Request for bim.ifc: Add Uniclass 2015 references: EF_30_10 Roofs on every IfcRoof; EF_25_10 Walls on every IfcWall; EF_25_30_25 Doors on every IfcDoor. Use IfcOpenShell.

First a look at what the model holds.

```python
import ifcopenshell

model = ifcopenshell.open("bim.ifc")
print(model.schema)
print("classifications:", [c.Name for c in model.by_type("IfcClassification")])
for ifc_class in ("IfcDoor", "IfcRoof", "IfcStair", "IfcWall", "IfcWindow"):
    print(ifc_class, len(model.by_type(ifc_class)))
```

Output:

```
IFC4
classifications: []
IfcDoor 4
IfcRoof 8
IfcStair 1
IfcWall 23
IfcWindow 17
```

```python
import ifcopenshell
import ifcopenshell.api.classification

model = ifcopenshell.open("bim.ifc")

system = ifcopenshell.api.classification.add_classification(model, classification="Uniclass 2015")

codes = {
    "IfcRoof": ("EF_30_10", "Roofs"),
    "IfcWall": ("EF_25_10", "Walls"),
    "IfcDoor": ("EF_25_30_25", "Doors"),
}
for ifc_class, (code, name) in codes.items():
    products = model.by_type(ifc_class)
    ifcopenshell.api.classification.add_reference(
        model, products=products, classification=system, identification=code, name=name
    )
    print(code, len(products))

model.write("bim_edited.ifc")
```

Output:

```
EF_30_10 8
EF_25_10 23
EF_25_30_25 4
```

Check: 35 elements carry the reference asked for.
